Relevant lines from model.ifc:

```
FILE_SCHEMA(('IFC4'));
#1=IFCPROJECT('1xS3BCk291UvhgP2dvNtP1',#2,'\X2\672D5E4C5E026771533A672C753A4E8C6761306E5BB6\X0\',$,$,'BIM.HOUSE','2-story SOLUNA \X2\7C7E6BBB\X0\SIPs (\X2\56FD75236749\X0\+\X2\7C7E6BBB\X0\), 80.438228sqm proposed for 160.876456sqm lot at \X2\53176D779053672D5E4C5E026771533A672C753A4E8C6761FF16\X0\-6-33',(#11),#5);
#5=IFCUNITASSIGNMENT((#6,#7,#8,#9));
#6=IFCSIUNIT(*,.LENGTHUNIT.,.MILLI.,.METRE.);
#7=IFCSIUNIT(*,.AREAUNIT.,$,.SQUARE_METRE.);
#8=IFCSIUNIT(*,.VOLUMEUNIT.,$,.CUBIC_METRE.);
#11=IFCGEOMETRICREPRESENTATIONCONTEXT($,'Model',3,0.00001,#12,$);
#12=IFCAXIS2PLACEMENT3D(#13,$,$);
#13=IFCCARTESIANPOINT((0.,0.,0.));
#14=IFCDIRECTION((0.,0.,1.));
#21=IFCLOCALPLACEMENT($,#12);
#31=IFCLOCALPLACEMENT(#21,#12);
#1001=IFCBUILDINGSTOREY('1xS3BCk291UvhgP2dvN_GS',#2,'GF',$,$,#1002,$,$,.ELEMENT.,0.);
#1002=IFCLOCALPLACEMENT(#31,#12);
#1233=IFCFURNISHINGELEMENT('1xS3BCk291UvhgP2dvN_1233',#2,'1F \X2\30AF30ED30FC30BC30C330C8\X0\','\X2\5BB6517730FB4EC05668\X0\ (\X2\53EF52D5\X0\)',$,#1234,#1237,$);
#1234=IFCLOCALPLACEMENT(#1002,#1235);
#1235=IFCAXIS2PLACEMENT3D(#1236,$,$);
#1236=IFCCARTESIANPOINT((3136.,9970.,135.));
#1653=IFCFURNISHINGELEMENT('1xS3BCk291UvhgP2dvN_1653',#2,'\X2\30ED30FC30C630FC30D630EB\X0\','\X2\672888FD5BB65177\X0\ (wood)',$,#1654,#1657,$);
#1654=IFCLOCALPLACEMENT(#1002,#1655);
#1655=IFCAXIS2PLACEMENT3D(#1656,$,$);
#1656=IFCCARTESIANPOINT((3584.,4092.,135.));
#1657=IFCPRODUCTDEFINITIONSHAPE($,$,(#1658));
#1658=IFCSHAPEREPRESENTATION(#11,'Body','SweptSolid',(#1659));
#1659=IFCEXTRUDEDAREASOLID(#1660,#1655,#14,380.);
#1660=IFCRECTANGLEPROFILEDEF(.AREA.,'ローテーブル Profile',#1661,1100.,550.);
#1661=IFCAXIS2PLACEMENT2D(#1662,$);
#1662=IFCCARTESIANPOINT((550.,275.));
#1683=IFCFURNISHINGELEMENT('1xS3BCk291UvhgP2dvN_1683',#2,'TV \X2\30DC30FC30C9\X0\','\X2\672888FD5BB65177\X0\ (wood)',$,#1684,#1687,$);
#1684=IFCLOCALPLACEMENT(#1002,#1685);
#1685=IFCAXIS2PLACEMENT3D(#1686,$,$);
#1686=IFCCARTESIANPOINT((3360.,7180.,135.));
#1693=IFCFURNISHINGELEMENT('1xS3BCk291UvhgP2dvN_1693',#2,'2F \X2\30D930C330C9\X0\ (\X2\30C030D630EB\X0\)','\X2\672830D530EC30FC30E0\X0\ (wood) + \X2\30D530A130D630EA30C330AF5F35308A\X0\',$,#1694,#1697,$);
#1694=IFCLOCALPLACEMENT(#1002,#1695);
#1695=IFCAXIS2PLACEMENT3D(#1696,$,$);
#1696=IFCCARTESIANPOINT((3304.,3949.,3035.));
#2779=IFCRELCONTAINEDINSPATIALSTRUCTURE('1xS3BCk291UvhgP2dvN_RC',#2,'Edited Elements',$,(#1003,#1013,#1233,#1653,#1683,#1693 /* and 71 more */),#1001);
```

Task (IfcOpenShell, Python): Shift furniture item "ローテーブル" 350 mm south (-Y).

```python
import ifcopenshell
import ifcopenshell.api.geometry
import ifcopenshell.util.placement

model = ifcopenshell.open("model.ifc")

item = model.by_id(1653)
matrix = ifcopenshell.util.placement.get_local_placement(item.ObjectPlacement)
matrix[1, 3] -= 350.0
ifcopenshell.api.geometry.edit_object_placement(model, product=item, matrix=matrix, is_si=False)

print(ifcopenshell.util.placement.get_local_placement(item.ObjectPlacement).round(3) + 0.0)

model.write("model_updated.ifc")
```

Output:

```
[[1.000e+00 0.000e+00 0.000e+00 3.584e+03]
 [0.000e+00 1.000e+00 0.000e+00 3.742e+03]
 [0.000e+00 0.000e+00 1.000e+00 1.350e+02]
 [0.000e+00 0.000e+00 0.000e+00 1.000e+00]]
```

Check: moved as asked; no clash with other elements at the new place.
